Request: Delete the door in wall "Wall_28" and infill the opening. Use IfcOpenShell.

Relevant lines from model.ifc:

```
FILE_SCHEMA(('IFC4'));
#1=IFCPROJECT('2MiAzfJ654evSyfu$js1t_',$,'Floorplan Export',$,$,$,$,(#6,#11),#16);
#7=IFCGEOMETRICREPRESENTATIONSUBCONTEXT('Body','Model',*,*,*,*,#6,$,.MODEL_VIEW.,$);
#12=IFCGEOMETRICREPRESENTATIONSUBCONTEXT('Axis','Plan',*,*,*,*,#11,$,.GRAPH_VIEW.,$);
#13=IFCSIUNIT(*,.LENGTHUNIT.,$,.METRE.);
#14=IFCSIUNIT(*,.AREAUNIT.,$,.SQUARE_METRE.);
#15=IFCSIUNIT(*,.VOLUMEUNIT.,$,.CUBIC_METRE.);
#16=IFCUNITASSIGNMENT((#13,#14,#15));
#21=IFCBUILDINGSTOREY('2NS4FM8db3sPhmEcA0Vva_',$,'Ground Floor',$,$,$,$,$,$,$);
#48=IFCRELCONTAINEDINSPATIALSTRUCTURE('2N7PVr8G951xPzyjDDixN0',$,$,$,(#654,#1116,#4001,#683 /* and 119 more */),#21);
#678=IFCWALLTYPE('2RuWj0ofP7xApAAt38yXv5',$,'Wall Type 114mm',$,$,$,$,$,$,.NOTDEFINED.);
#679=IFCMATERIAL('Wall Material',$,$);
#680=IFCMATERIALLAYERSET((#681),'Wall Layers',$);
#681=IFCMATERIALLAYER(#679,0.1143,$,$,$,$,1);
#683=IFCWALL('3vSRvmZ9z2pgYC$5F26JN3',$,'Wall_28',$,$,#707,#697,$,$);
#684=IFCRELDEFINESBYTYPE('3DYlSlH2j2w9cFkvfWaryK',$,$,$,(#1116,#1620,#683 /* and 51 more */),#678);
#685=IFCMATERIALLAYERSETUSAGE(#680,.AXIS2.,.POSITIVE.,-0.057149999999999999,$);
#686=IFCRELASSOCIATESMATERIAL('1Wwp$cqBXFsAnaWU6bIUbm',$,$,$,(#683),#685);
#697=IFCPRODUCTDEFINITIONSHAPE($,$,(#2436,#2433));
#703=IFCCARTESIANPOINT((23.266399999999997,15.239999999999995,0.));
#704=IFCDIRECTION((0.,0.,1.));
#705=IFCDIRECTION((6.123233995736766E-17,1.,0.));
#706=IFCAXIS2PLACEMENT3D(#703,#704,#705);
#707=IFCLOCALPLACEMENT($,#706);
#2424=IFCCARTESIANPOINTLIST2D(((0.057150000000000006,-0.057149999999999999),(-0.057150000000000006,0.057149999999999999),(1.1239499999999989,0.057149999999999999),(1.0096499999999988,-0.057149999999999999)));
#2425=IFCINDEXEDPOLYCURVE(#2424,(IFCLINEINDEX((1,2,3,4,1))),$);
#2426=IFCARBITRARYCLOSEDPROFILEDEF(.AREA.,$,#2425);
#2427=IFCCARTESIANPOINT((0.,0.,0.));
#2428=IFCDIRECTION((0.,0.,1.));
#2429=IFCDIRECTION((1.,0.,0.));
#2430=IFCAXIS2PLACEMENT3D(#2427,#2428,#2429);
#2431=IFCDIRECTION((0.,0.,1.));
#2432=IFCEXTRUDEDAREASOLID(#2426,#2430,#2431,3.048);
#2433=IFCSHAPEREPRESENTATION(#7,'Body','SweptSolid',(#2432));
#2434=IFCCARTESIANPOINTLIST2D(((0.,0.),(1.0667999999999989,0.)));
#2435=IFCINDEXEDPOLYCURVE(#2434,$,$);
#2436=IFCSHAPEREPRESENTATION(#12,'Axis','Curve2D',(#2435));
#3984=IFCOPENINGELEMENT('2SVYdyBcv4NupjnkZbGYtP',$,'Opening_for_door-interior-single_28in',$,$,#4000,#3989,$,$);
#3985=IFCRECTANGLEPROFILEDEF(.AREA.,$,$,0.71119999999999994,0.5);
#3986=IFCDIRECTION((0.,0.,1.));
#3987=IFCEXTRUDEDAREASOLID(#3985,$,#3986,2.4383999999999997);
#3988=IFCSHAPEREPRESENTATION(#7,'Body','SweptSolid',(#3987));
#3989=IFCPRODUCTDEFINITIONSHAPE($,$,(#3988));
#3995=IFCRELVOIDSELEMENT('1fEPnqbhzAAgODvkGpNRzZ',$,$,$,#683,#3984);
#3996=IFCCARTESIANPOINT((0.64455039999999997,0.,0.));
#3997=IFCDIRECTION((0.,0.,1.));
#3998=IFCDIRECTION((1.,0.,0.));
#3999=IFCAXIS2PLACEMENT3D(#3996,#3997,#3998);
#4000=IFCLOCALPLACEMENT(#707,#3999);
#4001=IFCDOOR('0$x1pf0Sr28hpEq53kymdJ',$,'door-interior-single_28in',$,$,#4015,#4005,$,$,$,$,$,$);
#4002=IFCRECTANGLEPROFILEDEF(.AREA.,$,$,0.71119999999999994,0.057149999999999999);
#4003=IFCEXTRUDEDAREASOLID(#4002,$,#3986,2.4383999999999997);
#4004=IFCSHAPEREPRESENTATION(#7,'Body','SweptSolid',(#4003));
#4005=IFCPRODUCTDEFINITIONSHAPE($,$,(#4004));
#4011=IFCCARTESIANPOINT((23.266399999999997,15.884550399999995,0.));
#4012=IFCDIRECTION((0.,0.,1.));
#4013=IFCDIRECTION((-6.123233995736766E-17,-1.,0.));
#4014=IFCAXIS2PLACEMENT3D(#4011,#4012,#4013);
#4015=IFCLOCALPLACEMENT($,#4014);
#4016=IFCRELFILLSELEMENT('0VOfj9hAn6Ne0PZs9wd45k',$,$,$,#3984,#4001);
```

```python
import ifcopenshell
import ifcopenshell.api.feature
import ifcopenshell.api.root
import ifcopenshell.geom
import ifcopenshell.util.shape

model = ifcopenshell.open("model.ifc")
settings = ifcopenshell.geom.settings()


def volume(element):
    """Net volume in cubic metres, openings subtracted."""
    shape = ifcopenshell.geom.create_shape(settings, element)
    return ifcopenshell.util.shape.get_volume(shape.geometry)


door = model.by_guid("0$x1pf0Sr28hpEq53kymdJ")
opening = door.FillsVoids[0].RelatingOpeningElement
wall = opening.VoidsElements[0].RelatingBuildingElement
before = volume(wall)

ifcopenshell.api.root.remove_product(model, product=door)
ifcopenshell.api.feature.remove_feature(model, feature=opening)

after = volume(wall)

print(f"wall volume {before:.3f} -> {after:.3f} m3")

model.write("model-out.ifc")
```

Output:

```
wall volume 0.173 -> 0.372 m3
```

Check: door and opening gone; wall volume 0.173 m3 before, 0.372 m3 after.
